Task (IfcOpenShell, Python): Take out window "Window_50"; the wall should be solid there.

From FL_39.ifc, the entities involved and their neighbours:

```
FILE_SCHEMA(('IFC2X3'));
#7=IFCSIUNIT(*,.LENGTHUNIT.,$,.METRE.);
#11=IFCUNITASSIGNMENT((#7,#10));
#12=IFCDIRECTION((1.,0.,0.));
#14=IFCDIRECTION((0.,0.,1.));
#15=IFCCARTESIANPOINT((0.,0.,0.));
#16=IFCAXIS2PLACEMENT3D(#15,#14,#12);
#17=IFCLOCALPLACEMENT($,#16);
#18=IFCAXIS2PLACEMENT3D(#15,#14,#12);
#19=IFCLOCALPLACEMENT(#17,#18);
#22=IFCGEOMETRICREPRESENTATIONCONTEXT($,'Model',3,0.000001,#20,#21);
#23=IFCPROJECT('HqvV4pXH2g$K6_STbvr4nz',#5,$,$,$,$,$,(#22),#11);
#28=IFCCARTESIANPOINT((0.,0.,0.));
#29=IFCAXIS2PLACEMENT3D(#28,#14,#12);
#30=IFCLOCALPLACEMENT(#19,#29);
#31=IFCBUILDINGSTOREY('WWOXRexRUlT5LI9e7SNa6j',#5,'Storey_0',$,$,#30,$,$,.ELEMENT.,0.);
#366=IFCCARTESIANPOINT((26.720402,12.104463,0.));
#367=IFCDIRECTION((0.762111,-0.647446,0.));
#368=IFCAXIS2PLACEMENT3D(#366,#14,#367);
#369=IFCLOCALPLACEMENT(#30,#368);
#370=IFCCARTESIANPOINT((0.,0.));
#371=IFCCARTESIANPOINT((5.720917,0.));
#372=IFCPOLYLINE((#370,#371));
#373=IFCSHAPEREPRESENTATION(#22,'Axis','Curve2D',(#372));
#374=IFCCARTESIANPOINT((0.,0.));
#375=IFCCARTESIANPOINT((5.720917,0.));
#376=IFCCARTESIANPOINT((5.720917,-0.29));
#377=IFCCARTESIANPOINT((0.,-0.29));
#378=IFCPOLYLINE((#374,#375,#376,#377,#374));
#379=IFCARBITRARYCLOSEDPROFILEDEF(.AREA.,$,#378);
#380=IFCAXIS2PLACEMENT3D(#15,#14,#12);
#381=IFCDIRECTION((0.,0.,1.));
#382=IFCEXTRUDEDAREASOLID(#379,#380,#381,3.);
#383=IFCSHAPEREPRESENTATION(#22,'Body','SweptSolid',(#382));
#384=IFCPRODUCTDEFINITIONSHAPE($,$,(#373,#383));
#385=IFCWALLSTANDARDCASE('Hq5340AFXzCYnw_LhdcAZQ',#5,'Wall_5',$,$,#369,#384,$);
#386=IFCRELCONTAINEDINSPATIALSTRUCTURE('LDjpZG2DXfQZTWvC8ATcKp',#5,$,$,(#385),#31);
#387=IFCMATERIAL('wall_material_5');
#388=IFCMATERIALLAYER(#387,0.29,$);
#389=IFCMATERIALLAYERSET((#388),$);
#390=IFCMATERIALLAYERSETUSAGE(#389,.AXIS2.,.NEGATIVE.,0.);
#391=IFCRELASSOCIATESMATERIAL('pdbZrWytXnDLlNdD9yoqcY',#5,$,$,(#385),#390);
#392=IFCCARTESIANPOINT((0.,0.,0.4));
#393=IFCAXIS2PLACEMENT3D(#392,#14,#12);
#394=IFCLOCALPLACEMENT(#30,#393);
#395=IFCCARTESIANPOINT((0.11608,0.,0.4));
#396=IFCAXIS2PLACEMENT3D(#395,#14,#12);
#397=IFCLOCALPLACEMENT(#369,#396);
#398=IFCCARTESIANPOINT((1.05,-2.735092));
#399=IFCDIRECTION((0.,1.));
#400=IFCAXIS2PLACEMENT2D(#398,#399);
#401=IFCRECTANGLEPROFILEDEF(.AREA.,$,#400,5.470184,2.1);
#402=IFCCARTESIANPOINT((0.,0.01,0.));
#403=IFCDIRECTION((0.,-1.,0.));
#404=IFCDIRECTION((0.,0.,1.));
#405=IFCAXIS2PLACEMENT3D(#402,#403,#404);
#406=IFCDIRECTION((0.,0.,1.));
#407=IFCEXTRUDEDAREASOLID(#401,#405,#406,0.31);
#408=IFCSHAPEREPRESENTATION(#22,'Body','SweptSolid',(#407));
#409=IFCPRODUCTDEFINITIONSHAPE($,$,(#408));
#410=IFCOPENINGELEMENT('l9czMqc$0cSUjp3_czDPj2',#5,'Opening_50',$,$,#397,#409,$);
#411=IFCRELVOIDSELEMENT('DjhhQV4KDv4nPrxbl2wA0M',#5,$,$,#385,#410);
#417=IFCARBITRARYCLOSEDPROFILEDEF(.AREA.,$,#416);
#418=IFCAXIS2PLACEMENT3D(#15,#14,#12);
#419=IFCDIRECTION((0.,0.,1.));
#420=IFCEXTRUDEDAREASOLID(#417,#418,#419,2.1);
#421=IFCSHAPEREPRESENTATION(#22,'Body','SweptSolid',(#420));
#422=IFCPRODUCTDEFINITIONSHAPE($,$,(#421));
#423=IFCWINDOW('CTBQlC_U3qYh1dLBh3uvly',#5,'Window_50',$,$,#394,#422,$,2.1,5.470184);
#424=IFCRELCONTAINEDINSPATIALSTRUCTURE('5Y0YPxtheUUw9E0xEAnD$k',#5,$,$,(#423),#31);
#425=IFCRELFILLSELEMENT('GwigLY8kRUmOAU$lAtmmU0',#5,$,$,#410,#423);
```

```python
import ifcopenshell
import ifcopenshell.api.feature
import ifcopenshell.api.root
import ifcopenshell.geom
import ifcopenshell.util.shape

model = ifcopenshell.open("FL_39.ifc")
settings = ifcopenshell.geom.settings()


def volume(element):
    """Net volume in cubic metres, openings subtracted."""
    shape = ifcopenshell.geom.create_shape(settings, element)
    return ifcopenshell.util.shape.get_volume(shape.geometry)


window = model.by_id(423)
opening = window.FillsVoids[0].RelatingOpeningElement
wall = opening.VoidsElements[0].RelatingBuildingElement
before = volume(wall)

ifcopenshell.api.root.remove_product(model, product=window)
ifcopenshell.api.feature.remove_feature(model, feature=opening)

after = volume(wall)

print(f"wall volume {before:.3f} -> {after:.3f} m3")

model.write("FL_39_rev.ifc")
```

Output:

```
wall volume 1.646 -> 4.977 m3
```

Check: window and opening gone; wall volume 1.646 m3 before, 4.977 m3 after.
